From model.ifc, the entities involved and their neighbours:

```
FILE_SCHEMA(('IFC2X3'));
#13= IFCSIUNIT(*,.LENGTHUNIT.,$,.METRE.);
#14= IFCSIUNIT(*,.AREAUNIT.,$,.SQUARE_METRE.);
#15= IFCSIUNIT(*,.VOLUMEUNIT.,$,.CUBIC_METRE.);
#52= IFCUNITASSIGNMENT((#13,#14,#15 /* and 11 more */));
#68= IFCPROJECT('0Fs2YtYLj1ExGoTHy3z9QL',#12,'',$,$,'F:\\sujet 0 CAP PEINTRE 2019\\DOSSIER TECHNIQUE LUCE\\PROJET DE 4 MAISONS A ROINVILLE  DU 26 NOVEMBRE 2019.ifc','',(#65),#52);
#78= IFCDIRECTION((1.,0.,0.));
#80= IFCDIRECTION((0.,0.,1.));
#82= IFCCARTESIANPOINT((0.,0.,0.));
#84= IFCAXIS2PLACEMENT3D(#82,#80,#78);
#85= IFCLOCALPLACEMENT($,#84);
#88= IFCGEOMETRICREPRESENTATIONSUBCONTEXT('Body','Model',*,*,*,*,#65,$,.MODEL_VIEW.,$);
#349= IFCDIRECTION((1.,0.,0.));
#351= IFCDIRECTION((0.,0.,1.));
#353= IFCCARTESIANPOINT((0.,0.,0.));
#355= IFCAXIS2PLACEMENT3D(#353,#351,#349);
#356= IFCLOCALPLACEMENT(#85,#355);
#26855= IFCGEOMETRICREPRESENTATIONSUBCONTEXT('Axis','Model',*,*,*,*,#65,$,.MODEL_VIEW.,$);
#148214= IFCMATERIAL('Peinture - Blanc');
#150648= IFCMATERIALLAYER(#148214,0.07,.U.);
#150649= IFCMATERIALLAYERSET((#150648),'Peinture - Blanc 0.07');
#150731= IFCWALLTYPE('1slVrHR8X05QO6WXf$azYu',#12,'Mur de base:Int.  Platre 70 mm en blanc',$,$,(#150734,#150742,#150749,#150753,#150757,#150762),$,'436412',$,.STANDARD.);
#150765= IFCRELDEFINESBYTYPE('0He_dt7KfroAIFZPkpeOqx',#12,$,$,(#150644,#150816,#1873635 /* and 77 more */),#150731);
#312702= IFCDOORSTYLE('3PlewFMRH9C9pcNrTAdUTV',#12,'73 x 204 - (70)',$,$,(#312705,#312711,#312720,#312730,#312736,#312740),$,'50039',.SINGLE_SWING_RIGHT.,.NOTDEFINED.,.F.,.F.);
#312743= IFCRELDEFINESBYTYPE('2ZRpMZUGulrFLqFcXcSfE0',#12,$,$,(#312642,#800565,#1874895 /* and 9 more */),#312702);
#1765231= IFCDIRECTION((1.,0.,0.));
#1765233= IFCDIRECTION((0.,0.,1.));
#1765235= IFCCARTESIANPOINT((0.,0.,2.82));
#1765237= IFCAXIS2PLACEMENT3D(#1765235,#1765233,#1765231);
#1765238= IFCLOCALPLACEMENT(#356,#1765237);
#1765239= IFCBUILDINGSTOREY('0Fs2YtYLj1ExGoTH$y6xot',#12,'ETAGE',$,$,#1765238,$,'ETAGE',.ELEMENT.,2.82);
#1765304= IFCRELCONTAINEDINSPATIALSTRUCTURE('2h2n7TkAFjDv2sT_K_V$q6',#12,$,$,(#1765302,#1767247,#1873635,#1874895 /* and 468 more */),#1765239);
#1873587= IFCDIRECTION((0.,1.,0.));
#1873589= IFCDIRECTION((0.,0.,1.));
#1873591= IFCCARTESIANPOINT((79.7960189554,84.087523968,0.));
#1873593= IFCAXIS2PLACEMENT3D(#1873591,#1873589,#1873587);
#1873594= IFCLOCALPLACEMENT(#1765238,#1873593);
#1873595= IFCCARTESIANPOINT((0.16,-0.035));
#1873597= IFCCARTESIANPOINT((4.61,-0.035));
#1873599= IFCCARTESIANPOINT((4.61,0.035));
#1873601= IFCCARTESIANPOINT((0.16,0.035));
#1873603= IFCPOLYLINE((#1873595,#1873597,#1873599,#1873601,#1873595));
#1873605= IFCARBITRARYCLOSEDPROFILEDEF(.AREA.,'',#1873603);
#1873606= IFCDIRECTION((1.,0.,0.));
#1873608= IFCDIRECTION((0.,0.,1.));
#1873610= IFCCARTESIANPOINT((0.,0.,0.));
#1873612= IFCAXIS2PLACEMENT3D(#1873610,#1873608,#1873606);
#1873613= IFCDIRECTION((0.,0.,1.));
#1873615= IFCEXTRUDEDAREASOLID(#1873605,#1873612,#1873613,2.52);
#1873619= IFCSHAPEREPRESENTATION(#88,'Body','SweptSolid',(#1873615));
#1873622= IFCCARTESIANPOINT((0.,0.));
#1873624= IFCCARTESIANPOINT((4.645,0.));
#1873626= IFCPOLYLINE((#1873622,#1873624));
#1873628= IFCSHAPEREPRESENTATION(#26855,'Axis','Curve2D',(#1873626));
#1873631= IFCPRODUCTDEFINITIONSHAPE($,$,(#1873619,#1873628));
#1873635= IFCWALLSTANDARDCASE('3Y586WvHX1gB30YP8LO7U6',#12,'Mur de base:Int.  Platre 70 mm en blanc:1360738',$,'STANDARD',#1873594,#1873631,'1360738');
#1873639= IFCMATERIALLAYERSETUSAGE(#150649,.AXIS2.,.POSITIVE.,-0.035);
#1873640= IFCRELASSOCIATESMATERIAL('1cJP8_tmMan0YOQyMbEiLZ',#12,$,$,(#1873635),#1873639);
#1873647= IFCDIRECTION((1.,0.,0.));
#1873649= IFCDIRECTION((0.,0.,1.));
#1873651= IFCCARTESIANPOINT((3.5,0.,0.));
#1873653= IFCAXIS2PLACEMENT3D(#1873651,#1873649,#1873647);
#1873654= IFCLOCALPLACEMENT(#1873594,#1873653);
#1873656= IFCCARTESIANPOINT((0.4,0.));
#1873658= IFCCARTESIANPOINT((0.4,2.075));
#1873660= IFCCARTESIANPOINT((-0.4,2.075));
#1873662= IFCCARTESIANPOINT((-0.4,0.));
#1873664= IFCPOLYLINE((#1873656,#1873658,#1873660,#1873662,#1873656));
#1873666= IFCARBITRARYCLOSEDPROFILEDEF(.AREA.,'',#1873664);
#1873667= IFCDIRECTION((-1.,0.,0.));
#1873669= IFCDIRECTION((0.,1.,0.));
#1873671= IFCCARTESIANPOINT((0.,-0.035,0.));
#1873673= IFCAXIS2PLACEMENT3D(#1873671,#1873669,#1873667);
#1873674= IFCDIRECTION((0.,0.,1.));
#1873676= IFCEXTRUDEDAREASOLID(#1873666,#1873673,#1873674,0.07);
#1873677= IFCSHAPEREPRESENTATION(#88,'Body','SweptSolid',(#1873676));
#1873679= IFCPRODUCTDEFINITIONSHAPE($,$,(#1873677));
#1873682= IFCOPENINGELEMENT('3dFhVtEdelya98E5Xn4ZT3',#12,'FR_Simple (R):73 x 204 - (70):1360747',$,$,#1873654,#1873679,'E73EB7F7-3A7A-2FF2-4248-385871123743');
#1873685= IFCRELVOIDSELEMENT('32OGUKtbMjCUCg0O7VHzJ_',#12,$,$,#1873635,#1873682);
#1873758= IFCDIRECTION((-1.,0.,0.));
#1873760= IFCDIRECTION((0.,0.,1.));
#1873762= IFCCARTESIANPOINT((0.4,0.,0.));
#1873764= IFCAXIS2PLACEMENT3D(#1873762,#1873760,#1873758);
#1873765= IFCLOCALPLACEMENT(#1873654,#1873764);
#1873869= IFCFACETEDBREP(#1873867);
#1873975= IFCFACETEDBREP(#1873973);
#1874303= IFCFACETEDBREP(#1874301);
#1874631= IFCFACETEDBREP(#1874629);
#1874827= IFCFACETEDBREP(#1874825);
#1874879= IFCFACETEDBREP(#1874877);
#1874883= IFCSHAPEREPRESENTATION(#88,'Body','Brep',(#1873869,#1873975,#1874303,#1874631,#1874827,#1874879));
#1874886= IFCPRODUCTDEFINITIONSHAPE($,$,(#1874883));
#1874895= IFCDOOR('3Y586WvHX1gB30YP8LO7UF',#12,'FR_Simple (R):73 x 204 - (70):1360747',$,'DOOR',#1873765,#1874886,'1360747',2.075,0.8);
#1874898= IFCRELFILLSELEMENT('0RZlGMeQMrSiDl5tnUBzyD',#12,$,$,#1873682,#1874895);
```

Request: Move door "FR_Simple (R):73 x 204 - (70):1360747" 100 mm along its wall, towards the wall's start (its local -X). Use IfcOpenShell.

```python
import ifcopenshell
import ifcopenshell.api.geometry
import ifcopenshell.util.placement

model = ifcopenshell.open("model.ifc")

door = model.by_guid("3Y586WvHX1gB30YP8LO7UF")
opening = door.FillsVoids[0].RelatingOpeningElement
wall = opening.VoidsElements[0].RelatingBuildingElement

wall_matrix = ifcopenshell.util.placement.get_local_placement(wall.ObjectPlacement)
shift = wall_matrix[:3, 0] * -0.1
before = ifcopenshell.util.placement.get_local_placement(door.ObjectPlacement)[:3, 3].copy()

# The door is placed relative to its opening, so it follows when the opening moves.
matrix = ifcopenshell.util.placement.get_local_placement(opening.ObjectPlacement)
matrix[:3, 3] += shift
ifcopenshell.api.geometry.edit_object_placement(
    model, product=opening, matrix=matrix, is_si=False, should_transform_children=True
)

after = ifcopenshell.util.placement.get_local_placement(door.ObjectPlacement)[:3, 3]
print("door moved by", (after - before).round(3) + 0.0)

model.write("model_edited.ifc")
```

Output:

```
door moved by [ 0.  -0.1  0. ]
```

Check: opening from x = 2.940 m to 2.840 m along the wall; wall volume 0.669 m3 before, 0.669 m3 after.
